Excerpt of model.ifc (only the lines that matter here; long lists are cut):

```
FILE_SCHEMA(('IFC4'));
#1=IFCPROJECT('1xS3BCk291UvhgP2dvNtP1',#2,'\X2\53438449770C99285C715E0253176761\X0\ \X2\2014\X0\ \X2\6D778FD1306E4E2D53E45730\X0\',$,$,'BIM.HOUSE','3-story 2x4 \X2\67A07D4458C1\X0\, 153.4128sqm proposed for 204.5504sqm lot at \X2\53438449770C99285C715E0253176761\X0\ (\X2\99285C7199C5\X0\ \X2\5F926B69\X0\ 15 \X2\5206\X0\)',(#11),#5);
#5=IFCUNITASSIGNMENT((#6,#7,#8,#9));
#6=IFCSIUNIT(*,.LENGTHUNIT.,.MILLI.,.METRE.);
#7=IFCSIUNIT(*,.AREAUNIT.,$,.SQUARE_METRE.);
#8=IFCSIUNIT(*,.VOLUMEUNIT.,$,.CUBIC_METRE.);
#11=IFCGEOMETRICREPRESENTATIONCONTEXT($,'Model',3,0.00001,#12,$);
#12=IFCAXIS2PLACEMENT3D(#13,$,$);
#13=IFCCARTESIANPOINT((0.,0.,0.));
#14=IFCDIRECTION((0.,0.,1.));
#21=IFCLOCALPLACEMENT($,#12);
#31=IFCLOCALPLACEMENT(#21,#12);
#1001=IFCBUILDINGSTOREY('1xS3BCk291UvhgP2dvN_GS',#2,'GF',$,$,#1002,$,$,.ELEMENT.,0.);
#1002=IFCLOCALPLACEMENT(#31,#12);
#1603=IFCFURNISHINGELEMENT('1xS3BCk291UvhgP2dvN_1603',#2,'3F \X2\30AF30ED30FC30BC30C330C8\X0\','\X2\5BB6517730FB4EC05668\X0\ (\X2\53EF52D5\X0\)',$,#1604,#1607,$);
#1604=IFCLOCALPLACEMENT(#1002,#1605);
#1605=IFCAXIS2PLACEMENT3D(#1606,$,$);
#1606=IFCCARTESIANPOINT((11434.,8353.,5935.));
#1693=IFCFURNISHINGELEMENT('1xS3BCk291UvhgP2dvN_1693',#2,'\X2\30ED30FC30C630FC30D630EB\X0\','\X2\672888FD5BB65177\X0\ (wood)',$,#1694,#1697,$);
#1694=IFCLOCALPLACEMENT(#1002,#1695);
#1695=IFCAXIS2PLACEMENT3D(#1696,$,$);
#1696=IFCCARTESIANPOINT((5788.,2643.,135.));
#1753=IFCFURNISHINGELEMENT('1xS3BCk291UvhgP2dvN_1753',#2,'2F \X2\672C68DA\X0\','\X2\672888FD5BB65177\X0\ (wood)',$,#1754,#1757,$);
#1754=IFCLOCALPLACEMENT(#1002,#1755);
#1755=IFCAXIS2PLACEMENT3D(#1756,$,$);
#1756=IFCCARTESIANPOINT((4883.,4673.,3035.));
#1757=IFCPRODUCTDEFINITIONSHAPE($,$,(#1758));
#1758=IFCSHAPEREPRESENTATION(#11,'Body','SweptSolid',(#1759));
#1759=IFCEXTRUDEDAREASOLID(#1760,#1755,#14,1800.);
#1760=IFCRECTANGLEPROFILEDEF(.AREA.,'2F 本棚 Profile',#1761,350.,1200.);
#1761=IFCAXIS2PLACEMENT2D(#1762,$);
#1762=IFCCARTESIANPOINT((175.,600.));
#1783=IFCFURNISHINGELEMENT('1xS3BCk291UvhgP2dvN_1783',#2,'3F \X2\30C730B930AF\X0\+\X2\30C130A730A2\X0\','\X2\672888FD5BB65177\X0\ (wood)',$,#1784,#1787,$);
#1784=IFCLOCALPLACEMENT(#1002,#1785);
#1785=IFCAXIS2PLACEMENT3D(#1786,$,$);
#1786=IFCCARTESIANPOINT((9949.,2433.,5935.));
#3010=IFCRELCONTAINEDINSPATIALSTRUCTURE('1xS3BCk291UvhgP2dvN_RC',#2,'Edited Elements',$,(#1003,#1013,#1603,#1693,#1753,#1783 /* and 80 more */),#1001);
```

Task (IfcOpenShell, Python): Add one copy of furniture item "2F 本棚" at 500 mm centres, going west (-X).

```python
import numpy as np
import ifcopenshell
import ifcopenshell.api.geometry
import ifcopenshell.api.root
import ifcopenshell.util.element
import ifcopenshell.util.placement

model = ifcopenshell.open("model.ifc")


def reuse_history(source, copy):
    """copy_class also copies each property set's owner history, people and application; keep the originals."""
    for rel in copy.IsDefinedBy:
        if rel.is_a("IfcRelDefinesByProperties") and (history := rel.RelatingPropertyDefinition.OwnerHistory):
            rel.RelatingPropertyDefinition.OwnerHistory = source.OwnerHistory
            ifcopenshell.util.element.remove_deep2(model, history)


source = model.by_id(1753)
base = ifcopenshell.util.placement.get_local_placement(source.ObjectPlacement)
step = np.array([-1.0, 0.0, 0.0]) * 500.0

for i in range(1, 2):
    copy = ifcopenshell.api.root.copy_class(model, product=source)
    copy.Representation = ifcopenshell.util.element.copy_deep(
        model, source.Representation, exclude=["IfcGeometricRepresentationContext", "IfcRepresentationMap"]
    )
    reuse_history(source, copy)
    matrix = base.copy()
    matrix[:3, 3] += i * step
    print("added at", matrix[:3, 3].round(3) + 0.0)
    ifcopenshell.api.geometry.edit_object_placement(model, product=copy, matrix=matrix, is_si=False)

model.write("model_rev.ifc")
```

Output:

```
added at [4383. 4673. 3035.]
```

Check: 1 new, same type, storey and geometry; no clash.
